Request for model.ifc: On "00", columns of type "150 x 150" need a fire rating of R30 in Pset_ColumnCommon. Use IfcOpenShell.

First a look at what the model holds.

```python
import ifcopenshell
import ifcopenshell.util.element

model = ifcopenshell.open("model.ifc")
print(model.schema)
storey = next(s for s in model.by_type("IfcBuildingStorey") if s.Name == "00")
columns = [e for e in ifcopenshell.util.element.get_decomposition(storey) if e.is_a("IfcColumn")]
seen = {}
for e in columns:
    element_type = ifcopenshell.util.element.get_type(e)
    key = (element_type.Name if element_type != e and element_type else None, ifcopenshell.util.element.get_pset(e, "Pset_ColumnCommon", "FireRating"))
    seen[key] = seen.get(key, 0) + 1
for (name, value), count in sorted(seen.items(), key=str):
    print(count, "x", name, "|", value)
```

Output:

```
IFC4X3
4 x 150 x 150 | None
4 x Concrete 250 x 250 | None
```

```python
import ifcopenshell
import ifcopenshell.api.pset
import ifcopenshell.util.element

model = ifcopenshell.open("model.ifc")

storey = next(s for s in model.by_type("IfcBuildingStorey") if s.Name == "00")
columns = [e for e in ifcopenshell.util.element.get_decomposition(storey) if e.is_a("IfcColumn")]

count = 0
for e in columns:
    element_type = ifcopenshell.util.element.get_type(e)
    if element_type in (None, e) or element_type.Name != "150 x 150":
        continue
    # add_pset returns the element's existing set when there is one.
    pset = ifcopenshell.api.pset.add_pset(model, product=e, name="Pset_ColumnCommon")
    ifcopenshell.api.pset.edit_pset(model, pset=pset, properties={"FireRating": "R30"})
    count += 1

print(count, "columns updated")

model.write("model_rev.ifc")
```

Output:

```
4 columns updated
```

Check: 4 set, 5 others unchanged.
